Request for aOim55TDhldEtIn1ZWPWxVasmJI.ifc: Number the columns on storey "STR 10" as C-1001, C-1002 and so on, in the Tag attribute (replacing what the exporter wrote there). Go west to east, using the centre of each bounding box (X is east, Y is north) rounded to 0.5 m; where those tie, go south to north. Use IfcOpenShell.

First a look at what the model holds.

```python
import ifcopenshell
import ifcopenshell.util.element
import ifcopenshell.util.placement

model = ifcopenshell.open("aOim55TDhldEtIn1ZWPWxVasmJI.ifc")
print(model.schema)
storey = next(s for s in model.by_type("IfcBuildingStorey") if s.Name == "STR 10")
columns = [e for e in ifcopenshell.util.element.get_decomposition(storey) if e.is_a("IfcColumn")]
for e in sorted(columns, key=lambda e: e.id()):
    origin = ifcopenshell.util.placement.get_local_placement(e.ObjectPlacement)[:3, 3]
    print(e.id(), e.Tag, e.Name, origin.round(2) + 0.0, sep=" | ")
```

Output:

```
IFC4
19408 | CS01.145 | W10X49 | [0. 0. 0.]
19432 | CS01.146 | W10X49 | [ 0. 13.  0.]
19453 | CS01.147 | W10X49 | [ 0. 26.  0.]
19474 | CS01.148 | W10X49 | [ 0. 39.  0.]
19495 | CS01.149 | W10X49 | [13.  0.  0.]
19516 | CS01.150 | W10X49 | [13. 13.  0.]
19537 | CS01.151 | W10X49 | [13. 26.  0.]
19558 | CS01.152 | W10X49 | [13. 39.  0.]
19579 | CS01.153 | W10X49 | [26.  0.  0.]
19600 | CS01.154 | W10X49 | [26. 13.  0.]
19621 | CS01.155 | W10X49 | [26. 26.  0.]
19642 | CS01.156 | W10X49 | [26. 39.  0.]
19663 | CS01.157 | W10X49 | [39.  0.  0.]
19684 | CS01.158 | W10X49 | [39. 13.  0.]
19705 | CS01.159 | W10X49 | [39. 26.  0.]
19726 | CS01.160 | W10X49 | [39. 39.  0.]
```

```python
import ifcopenshell
import ifcopenshell.geom
import ifcopenshell.util.element
import ifcopenshell.util.shape

model = ifcopenshell.open("aOim55TDhldEtIn1ZWPWxVasmJI.ifc")
settings = ifcopenshell.geom.settings()
settings.set("use-world-coords", True)


def centre(element):
    shape = ifcopenshell.geom.create_shape(settings, element)
    return ifcopenshell.util.shape.get_bbox_centroid(shape.geometry)


storey = next(s for s in model.by_type("IfcBuildingStorey") if s.Name == "STR 10")
columns = [e for e in ifcopenshell.util.element.get_decomposition(storey) if e.is_a("IfcColumn")]

# Insertion points can sit at a corner or the storey origin, so sort by the geometry (in metres).
centres = {e: centre(e) for e in columns}
columns.sort(key=lambda e: (round(centres[e][0] / 0.5), centres[e][1]))

for i, e in enumerate(columns, start=1):
    number = f"C-10{i:02d}"
    e.Tag = number
    print(e.id(), number)

model.write("aOim55TDhldEtIn1ZWPWxVasmJI_v2.ifc")
```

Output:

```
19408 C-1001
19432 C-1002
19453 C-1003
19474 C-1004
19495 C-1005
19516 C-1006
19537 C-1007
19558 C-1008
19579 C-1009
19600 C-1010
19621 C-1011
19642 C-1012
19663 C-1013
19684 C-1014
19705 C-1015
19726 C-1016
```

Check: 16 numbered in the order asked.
